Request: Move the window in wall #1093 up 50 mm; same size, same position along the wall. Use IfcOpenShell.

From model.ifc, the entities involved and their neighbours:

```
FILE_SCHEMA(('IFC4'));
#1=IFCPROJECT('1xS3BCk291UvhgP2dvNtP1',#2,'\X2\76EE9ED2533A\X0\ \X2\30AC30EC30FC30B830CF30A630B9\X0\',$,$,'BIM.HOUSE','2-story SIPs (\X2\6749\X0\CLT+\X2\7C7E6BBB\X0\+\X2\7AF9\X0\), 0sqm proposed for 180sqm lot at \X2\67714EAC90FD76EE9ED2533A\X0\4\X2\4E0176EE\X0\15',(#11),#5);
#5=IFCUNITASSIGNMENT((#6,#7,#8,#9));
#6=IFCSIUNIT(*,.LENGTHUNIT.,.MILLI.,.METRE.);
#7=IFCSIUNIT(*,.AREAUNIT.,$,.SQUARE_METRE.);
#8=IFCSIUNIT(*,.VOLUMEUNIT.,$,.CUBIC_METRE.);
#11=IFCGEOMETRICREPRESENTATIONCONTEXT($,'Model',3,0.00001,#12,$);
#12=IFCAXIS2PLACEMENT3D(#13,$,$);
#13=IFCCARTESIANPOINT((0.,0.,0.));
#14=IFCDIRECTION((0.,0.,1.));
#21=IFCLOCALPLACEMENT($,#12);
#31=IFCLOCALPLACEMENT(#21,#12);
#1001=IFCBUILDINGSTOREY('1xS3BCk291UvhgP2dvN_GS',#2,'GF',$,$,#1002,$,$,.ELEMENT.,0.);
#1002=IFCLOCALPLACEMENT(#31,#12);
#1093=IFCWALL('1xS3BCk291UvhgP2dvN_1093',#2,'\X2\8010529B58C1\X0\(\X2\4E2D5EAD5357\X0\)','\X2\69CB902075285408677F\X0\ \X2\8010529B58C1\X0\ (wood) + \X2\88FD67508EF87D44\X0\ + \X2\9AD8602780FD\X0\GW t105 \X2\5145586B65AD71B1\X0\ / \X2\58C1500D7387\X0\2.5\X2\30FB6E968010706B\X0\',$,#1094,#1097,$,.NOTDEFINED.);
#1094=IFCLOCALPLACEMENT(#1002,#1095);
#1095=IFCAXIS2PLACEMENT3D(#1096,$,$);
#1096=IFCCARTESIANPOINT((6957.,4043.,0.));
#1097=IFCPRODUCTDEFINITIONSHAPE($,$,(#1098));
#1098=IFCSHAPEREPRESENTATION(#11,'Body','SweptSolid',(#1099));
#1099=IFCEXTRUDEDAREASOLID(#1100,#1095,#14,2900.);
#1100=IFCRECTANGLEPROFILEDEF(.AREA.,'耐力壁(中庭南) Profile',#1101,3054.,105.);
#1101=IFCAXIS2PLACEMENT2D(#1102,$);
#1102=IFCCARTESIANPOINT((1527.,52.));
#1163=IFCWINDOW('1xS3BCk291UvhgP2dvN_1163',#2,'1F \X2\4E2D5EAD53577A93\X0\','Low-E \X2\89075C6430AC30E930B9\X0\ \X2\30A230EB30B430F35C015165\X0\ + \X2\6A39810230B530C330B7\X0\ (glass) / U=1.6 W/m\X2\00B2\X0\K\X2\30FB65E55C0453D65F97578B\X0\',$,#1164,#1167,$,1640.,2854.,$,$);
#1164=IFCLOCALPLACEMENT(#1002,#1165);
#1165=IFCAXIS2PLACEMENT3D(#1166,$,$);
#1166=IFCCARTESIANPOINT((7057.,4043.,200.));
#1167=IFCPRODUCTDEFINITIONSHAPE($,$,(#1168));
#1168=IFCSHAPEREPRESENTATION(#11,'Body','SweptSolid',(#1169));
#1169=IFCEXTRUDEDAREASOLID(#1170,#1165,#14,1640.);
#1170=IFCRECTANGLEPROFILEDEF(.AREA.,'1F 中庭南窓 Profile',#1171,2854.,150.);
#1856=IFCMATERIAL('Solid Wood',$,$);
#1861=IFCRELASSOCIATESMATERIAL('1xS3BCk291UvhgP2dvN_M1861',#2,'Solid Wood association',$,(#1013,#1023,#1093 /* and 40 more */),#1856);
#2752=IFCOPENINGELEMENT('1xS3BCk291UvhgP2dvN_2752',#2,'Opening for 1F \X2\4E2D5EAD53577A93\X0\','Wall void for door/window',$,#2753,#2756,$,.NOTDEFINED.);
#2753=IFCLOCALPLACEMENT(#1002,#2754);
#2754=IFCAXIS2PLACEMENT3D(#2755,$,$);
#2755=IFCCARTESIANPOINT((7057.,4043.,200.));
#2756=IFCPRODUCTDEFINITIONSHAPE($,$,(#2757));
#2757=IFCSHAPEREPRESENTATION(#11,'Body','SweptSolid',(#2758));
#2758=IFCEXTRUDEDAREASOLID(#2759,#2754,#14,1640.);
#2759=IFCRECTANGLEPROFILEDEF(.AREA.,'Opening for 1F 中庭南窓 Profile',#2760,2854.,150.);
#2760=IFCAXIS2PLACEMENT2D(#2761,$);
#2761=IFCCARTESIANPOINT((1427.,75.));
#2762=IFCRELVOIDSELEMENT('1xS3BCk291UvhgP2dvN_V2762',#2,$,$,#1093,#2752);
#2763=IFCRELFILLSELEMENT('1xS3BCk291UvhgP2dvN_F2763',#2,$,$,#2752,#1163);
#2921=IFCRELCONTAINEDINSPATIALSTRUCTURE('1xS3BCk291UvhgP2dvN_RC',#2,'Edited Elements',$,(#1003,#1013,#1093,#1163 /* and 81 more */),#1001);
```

```python
import numpy as np
import ifcopenshell
import ifcopenshell.api.geometry
import ifcopenshell.util.placement
import ifcopenshell.util.unit

model = ifcopenshell.open("model.ifc")
unit_scale = ifcopenshell.util.unit.calculate_unit_scale(model)

window = model.by_guid("1xS3BCk291UvhgP2dvN_1163")
opening = window.FillsVoids[0].RelatingOpeningElement
dz = 0.05 / unit_scale

shift = np.array([0.0, 0.0, dz])
# The window is not placed relative to its opening, so move both.
for product in (opening, window):
    matrix = ifcopenshell.util.placement.get_local_placement(product.ObjectPlacement)
    matrix[:3, 3] += shift
    ifcopenshell.api.geometry.edit_object_placement(model, product=product, matrix=matrix, is_si=False)

print(f"moved by {dz * unit_scale:+.3f} m")

model.write("model_updated.ifc")
```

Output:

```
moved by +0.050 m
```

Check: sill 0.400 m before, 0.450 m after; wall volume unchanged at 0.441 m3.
